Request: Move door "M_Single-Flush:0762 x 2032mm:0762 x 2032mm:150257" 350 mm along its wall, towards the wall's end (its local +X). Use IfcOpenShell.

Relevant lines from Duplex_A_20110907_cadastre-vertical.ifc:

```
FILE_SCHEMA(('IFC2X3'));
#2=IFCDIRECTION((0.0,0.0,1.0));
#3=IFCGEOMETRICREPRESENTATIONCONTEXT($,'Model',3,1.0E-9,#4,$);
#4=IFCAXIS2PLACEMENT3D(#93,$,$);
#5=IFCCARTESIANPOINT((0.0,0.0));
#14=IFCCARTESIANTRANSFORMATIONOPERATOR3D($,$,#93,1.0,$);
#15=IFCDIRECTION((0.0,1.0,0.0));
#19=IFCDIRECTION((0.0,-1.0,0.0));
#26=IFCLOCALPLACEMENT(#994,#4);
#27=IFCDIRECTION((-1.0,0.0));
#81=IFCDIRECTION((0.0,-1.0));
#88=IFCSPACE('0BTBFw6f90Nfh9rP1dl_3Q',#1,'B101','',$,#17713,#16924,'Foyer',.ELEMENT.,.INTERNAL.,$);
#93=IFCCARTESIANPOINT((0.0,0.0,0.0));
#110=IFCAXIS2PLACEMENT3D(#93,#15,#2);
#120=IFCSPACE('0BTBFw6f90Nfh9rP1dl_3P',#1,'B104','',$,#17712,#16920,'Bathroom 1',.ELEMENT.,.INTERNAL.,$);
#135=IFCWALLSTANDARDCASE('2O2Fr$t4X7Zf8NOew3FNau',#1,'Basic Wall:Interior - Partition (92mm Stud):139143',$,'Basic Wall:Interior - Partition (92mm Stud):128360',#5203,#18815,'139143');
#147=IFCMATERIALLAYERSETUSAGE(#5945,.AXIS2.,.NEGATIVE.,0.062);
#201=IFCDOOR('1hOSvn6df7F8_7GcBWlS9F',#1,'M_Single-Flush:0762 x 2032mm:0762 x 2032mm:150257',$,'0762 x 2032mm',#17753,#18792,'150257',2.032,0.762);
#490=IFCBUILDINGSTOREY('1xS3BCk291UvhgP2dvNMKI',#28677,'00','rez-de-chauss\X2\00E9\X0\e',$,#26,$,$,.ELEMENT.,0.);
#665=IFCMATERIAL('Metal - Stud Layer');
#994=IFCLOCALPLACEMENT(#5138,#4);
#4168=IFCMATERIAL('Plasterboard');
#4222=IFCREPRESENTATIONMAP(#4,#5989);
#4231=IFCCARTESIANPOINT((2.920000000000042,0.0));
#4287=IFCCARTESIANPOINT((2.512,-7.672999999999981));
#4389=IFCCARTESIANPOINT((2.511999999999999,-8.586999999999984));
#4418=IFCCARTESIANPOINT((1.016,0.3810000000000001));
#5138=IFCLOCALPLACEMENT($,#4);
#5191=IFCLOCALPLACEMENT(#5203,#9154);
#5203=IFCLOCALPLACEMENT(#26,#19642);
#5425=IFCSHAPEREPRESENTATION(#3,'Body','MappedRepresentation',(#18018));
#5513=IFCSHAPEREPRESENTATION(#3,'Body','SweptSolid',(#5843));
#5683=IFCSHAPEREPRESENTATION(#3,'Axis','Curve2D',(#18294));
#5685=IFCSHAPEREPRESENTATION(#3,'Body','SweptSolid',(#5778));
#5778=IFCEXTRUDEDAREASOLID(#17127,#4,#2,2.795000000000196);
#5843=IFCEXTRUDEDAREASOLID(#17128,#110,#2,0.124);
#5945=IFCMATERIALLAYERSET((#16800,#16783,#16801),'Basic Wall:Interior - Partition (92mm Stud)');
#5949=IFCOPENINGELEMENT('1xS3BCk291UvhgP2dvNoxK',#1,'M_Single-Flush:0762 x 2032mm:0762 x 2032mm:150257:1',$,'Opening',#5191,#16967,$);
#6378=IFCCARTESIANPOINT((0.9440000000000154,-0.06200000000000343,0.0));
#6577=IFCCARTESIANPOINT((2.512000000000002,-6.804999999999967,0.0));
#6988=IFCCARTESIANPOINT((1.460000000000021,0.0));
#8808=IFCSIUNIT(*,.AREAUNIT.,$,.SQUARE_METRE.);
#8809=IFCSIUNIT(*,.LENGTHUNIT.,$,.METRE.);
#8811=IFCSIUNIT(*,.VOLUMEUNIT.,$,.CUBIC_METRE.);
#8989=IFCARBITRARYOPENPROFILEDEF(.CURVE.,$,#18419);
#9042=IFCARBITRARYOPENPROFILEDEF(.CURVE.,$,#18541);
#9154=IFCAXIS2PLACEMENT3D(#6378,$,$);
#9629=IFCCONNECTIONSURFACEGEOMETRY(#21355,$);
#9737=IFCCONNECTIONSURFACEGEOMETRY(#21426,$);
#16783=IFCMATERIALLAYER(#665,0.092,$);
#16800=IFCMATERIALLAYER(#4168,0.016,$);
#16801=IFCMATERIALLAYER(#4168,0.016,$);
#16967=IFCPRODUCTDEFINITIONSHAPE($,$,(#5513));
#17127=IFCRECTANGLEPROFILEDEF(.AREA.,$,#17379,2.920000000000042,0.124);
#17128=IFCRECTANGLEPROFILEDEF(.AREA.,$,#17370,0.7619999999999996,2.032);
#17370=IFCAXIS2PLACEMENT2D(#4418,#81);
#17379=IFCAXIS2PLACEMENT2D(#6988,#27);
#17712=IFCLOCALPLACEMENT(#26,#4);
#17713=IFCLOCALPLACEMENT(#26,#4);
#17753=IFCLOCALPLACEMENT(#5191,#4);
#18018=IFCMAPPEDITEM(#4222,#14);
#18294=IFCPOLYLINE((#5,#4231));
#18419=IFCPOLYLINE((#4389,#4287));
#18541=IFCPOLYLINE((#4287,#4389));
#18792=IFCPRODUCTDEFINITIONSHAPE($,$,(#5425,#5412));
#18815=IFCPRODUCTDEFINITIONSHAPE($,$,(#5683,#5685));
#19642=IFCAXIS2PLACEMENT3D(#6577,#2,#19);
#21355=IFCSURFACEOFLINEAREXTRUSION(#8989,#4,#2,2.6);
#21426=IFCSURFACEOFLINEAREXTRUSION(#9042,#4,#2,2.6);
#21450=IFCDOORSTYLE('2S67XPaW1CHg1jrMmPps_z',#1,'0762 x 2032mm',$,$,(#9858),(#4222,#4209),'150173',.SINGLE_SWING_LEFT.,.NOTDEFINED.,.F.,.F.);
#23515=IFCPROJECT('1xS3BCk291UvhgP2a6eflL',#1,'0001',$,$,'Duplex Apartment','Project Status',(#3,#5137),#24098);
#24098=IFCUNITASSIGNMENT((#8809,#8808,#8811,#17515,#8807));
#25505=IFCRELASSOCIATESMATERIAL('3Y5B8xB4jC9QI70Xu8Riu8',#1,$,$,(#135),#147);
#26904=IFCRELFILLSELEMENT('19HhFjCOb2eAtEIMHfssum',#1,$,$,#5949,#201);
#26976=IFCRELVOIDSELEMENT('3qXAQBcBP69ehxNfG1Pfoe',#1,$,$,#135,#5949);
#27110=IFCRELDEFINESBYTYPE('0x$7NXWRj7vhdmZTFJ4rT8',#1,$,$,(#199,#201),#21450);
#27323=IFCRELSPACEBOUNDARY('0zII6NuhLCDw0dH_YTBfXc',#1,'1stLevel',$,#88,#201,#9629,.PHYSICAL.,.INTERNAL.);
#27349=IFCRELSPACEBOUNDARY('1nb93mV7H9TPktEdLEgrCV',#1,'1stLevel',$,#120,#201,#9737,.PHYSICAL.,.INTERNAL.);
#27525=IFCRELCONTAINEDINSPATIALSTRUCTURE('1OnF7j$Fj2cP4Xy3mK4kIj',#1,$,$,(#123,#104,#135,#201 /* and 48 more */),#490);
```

```python
import numpy as np
import ifcopenshell
import ifcopenshell.api.geometry
import ifcopenshell.util.placement
import ifcopenshell.util.unit

model = ifcopenshell.open("Duplex_A_20110907_cadastre-vertical.ifc")
unit_scale = ifcopenshell.util.unit.calculate_unit_scale(model)

door = model.by_guid("1hOSvn6df7F8_7GcBWlS9F")
opening = door.FillsVoids[0].RelatingOpeningElement
wall = opening.VoidsElements[0].RelatingBuildingElement

wall_matrix = ifcopenshell.util.placement.get_local_placement(wall.ObjectPlacement)
shift = wall_matrix[:3, 0] * 0.35 / unit_scale
before = ifcopenshell.util.placement.get_local_placement(door.ObjectPlacement)[:3, 3].copy()

# The door is placed relative to its opening, so it follows when the opening moves.
matrix = ifcopenshell.util.placement.get_local_placement(opening.ObjectPlacement)
matrix[:3, 3] += shift
ifcopenshell.api.geometry.edit_object_placement(
    model, product=opening, matrix=matrix, is_si=False, should_transform_children=True
)

# Space boundary surfaces are stored in each space's coordinates; move them too.
for rel in door.ProvidesBoundaries:
    if not rel.ConnectionGeometry:
        continue
    surface = rel.ConnectionGeometry.SurfaceOnRelatingElement
    space_matrix = ifcopenshell.util.placement.get_local_placement(rel.RelatingSpace.ObjectPlacement)
    point = np.array(surface.Position.Location.Coordinates) + space_matrix[:3, :3].T @ shift
    surface.Position = model.createIfcAxis2Placement3D(
        model.createIfcCartesianPoint(point.tolist()), surface.Position.Axis, surface.Position.RefDirection
    )

after = ifcopenshell.util.placement.get_local_placement(door.ObjectPlacement)[:3, 3]
print("door moved by", (after - before).round(3) + 0.0)

model.write("Duplex_A_20110907_cadastre-vertical_edited.ifc")
```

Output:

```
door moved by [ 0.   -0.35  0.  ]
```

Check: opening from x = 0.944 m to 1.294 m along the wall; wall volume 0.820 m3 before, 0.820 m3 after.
